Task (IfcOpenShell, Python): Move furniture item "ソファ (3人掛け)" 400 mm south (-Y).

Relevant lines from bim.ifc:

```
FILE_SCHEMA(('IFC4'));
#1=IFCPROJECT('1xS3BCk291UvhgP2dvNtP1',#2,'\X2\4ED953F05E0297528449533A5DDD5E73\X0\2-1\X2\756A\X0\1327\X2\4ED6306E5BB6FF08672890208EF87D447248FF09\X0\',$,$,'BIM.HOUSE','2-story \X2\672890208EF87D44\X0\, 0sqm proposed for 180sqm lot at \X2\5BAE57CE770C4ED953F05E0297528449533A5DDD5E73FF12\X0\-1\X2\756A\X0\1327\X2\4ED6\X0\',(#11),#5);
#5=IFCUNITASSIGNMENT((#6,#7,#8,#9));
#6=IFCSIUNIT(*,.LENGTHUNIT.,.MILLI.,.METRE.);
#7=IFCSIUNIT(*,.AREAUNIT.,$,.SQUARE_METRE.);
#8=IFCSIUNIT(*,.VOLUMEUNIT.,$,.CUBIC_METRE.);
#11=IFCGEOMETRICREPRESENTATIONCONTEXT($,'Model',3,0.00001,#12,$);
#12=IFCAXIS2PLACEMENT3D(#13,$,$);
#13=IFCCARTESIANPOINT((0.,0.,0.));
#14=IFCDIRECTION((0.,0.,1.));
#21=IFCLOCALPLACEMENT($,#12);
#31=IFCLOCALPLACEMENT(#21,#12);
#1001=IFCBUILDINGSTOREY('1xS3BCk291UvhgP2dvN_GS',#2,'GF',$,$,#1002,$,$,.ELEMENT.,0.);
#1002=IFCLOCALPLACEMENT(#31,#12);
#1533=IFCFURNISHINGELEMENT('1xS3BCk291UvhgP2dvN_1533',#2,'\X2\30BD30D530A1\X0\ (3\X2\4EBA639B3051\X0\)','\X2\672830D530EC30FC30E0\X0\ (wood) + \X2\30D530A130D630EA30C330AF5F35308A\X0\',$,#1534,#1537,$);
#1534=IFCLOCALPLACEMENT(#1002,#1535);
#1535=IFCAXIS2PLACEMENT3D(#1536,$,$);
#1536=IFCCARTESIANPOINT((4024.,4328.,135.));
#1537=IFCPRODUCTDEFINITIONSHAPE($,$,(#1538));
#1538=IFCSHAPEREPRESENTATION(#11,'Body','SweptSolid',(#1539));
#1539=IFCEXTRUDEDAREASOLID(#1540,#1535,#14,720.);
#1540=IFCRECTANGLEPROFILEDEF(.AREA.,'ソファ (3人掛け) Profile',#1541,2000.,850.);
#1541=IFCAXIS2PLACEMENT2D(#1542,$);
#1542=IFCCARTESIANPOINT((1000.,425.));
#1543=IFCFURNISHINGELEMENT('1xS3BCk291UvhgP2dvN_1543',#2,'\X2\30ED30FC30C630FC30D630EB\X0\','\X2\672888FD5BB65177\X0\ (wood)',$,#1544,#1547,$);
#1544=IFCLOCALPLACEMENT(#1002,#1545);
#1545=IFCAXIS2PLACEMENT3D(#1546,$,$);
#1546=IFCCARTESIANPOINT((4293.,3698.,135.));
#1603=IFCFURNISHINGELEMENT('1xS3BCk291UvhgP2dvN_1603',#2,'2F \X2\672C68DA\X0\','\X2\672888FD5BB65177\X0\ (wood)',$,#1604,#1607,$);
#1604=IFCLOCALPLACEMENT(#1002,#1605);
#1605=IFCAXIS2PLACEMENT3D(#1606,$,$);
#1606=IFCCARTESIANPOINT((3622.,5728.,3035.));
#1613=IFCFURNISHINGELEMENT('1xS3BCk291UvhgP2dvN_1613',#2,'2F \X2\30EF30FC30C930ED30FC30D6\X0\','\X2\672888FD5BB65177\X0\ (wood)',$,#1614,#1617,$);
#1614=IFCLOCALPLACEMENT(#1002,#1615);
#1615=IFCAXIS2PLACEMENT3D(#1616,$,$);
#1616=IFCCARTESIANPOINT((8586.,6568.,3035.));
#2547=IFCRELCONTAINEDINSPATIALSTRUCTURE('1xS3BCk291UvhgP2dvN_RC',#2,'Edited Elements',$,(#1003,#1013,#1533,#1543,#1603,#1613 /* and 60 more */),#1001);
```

```python
import ifcopenshell
import ifcopenshell.api.geometry
import ifcopenshell.util.placement
import ifcopenshell.util.unit

model = ifcopenshell.open("bim.ifc")
unit_scale = ifcopenshell.util.unit.calculate_unit_scale(model)

item = model.by_guid("1xS3BCk291UvhgP2dvN_1533")
matrix = ifcopenshell.util.placement.get_local_placement(item.ObjectPlacement)
matrix[1, 3] -= 0.4 / unit_scale
ifcopenshell.api.geometry.edit_object_placement(model, product=item, matrix=matrix, is_si=False)

print(ifcopenshell.util.placement.get_local_placement(item.ObjectPlacement).round(3) + 0.0)

model.write("bim_rev.ifc")
```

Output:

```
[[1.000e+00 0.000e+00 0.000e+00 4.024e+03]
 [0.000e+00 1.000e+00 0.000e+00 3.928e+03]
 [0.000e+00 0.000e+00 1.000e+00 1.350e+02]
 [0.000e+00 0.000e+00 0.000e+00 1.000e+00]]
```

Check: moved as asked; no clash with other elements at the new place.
